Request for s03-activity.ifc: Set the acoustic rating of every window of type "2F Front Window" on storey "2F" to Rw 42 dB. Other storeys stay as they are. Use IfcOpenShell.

First a look at what the model holds.

```python
import ifcopenshell
import ifcopenshell.util.element

model = ifcopenshell.open("s03-activity.ifc")
print(model.schema)
storey = next(s for s in model.by_type("IfcBuildingStorey") if s.Name == "2F")
windows = [e for e in ifcopenshell.util.element.get_decomposition(storey) if e.is_a("IfcWindow")]
seen = {}
for e in windows:
    element_type = ifcopenshell.util.element.get_type(e)
    key = (element_type.Name if element_type != e and element_type else None, ifcopenshell.util.element.get_pset(e, "Pset_WindowCommon", "AcousticRating"))
    seen[key] = seen.get(key, 0) + 1
for (name, value), count in sorted(seen.items(), key=str):
    print(count, "x", name, "|", value)
```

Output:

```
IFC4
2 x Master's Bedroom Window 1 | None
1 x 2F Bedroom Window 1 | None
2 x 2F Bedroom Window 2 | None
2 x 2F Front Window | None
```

```python
import ifcopenshell
import ifcopenshell.api.pset
import ifcopenshell.util.element

model = ifcopenshell.open("s03-activity.ifc")

storey = next(s for s in model.by_type("IfcBuildingStorey") if s.Name == "2F")
windows = [e for e in ifcopenshell.util.element.get_decomposition(storey) if e.is_a("IfcWindow")]

count = 0
for e in windows:
    element_type = ifcopenshell.util.element.get_type(e)
    if element_type in (None, e) or element_type.Name != "2F Front Window":
        continue
    # add_pset returns the element's existing set when there is one.
    pset = ifcopenshell.api.pset.add_pset(model, product=e, name="Pset_WindowCommon")
    ifcopenshell.api.pset.edit_pset(model, pset=pset, properties={"AcousticRating": "Rw 42 dB"})
    count += 1

print(count, "windows updated")

model.write("s03-activity_v2.ifc")
```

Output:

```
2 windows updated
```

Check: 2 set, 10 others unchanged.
